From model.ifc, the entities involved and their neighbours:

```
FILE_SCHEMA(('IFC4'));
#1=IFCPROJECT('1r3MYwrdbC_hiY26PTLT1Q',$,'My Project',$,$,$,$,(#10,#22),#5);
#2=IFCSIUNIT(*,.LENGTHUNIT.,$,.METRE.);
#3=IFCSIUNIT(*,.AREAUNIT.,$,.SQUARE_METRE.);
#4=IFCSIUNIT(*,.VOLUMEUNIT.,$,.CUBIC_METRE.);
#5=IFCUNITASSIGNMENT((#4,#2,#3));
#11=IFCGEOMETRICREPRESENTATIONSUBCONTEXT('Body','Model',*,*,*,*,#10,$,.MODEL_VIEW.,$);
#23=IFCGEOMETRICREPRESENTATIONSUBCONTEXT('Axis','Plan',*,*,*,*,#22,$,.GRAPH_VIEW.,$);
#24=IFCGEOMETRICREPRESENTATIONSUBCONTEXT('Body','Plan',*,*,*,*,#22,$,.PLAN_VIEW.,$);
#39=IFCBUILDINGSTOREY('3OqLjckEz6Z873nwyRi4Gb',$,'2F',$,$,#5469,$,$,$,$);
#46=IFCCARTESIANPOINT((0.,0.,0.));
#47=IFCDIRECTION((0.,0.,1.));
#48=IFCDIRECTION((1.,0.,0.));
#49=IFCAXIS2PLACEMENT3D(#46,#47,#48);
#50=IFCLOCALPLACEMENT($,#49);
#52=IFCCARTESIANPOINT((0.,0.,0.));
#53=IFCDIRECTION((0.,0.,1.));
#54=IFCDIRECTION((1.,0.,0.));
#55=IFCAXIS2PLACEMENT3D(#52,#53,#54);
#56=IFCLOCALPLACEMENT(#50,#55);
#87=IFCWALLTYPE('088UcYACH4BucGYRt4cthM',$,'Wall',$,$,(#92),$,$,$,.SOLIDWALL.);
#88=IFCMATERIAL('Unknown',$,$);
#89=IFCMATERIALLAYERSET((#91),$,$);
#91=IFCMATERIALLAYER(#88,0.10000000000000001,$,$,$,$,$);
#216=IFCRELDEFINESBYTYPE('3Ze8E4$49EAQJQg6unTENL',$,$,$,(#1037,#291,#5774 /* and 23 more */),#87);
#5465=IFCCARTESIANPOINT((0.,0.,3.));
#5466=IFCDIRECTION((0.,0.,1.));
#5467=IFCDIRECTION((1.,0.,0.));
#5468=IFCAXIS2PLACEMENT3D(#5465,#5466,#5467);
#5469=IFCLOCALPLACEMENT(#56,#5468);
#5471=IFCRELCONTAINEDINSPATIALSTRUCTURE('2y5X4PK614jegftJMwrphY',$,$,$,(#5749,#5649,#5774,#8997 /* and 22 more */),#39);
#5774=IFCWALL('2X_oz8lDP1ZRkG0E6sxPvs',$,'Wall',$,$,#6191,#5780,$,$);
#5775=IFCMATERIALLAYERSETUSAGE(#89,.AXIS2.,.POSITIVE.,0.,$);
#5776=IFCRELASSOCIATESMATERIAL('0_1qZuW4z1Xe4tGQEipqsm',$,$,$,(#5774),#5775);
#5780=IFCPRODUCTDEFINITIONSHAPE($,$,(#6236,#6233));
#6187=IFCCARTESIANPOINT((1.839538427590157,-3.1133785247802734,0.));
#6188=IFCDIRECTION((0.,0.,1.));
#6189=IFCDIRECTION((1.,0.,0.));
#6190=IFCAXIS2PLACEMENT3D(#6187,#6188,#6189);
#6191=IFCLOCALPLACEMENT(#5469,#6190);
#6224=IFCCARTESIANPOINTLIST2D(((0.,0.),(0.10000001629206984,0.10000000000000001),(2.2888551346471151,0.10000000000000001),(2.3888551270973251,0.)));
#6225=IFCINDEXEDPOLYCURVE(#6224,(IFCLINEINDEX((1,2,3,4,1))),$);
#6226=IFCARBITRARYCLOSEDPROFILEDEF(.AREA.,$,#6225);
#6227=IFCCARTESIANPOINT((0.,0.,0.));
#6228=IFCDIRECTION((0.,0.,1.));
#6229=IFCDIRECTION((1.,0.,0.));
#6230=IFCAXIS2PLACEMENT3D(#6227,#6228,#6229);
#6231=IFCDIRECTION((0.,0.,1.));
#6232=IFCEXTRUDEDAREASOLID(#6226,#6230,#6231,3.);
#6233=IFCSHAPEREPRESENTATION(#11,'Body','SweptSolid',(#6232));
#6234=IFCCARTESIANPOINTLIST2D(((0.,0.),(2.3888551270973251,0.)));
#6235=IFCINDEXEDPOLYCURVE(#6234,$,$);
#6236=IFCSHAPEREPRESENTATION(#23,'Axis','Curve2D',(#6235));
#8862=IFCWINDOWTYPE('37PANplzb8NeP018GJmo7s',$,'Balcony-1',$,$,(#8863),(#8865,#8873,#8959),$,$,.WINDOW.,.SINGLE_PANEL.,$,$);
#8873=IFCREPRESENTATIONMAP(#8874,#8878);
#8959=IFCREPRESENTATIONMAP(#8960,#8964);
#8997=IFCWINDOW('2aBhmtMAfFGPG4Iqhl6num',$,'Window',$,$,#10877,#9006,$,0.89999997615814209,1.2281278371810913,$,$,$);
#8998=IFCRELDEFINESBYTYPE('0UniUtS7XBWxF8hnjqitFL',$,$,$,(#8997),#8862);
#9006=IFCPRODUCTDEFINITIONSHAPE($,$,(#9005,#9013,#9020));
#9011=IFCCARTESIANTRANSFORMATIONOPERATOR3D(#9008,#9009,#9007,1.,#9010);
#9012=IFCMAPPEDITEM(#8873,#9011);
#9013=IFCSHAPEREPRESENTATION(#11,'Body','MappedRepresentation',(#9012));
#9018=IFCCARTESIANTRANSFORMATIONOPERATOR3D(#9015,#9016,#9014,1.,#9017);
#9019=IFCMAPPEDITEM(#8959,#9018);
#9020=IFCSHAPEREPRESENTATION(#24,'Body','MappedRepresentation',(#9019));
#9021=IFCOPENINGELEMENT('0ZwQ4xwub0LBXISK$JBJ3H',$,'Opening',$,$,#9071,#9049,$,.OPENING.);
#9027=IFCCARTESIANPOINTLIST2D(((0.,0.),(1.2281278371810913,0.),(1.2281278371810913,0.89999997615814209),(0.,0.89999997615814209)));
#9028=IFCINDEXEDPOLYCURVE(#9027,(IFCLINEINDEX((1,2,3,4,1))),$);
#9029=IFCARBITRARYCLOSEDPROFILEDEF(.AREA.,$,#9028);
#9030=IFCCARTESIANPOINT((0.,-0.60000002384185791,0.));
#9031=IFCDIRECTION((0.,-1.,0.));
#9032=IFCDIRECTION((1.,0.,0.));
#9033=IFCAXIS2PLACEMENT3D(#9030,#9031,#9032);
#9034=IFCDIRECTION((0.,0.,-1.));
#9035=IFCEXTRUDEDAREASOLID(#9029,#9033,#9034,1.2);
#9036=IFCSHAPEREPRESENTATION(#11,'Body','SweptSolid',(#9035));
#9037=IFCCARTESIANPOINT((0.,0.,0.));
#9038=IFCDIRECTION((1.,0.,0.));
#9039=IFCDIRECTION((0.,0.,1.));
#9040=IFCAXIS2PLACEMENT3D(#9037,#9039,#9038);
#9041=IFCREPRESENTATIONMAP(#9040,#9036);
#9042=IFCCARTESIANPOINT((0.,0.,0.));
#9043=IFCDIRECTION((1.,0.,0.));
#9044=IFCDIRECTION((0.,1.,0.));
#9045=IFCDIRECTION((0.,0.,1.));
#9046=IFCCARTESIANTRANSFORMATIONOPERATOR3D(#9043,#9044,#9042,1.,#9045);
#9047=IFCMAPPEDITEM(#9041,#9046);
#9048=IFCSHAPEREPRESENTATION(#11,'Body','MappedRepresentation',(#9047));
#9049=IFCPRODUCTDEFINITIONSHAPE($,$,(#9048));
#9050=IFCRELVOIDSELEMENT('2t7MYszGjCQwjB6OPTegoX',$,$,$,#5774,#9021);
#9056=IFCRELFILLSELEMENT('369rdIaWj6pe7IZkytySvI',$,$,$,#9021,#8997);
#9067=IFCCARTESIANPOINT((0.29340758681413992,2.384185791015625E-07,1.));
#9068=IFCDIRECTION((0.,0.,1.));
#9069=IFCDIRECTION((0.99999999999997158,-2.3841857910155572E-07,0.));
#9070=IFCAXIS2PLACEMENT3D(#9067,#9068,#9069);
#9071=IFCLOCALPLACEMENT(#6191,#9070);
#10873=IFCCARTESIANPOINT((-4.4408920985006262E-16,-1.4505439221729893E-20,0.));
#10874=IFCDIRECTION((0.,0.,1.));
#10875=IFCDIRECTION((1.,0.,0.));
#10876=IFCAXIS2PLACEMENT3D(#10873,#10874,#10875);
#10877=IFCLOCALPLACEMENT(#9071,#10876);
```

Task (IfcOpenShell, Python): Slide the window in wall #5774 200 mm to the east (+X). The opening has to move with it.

```python
import ifcopenshell
import ifcopenshell.api.geometry
import ifcopenshell.util.placement
import ifcopenshell.util.unit

model = ifcopenshell.open("model.ifc")
unit_scale = ifcopenshell.util.unit.calculate_unit_scale(model)

window = model.by_guid("2aBhmtMAfFGPG4Iqhl6num")
opening = window.FillsVoids[0].RelatingOpeningElement
wall = opening.VoidsElements[0].RelatingBuildingElement

wall_matrix = ifcopenshell.util.placement.get_local_placement(wall.ObjectPlacement)
shift = wall_matrix[:3, 0] * 0.2 / unit_scale
before = ifcopenshell.util.placement.get_local_placement(window.ObjectPlacement)[:3, 3].copy()

# The window is placed relative to its opening, so it follows when the opening moves.
matrix = ifcopenshell.util.placement.get_local_placement(opening.ObjectPlacement)
matrix[:3, 3] += shift
ifcopenshell.api.geometry.edit_object_placement(
    model, product=opening, matrix=matrix, is_si=False, should_transform_children=True
)

after = ifcopenshell.util.placement.get_local_placement(window.ObjectPlacement)[:3, 3]
print("window moved by", (after - before).round(3) + 0.0)

model.write("model-out.ifc")
```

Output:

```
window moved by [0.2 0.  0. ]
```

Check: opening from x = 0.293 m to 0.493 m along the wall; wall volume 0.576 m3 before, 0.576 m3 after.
